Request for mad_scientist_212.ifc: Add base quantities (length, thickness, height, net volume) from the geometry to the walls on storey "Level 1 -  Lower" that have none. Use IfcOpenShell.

First a look at what the model holds.

```python
import ifcopenshell
import ifcopenshell.util.element
import ifcopenshell.util.unit

model = ifcopenshell.open("mad_scientist_212.ifc")
print(model.schema)
for unit_type in ("LENGTHUNIT", "AREAUNIT", "VOLUMEUNIT"):
    print(unit_type, ifcopenshell.util.unit.calculate_unit_scale(model, unit_type))
storey = next(s for s in model.by_type("IfcBuildingStorey") if s.Name == "Level 1 -  Lower")
walls = [e for e in ifcopenshell.util.element.get_decomposition(storey) if e.is_a("IfcWall")]
for e in sorted(walls, key=lambda e: e.id()):
    print(e.id(), e.is_a(), e.Name, list(ifcopenshell.util.element.get_psets(e, qtos_only=True)), sep=" | ")
```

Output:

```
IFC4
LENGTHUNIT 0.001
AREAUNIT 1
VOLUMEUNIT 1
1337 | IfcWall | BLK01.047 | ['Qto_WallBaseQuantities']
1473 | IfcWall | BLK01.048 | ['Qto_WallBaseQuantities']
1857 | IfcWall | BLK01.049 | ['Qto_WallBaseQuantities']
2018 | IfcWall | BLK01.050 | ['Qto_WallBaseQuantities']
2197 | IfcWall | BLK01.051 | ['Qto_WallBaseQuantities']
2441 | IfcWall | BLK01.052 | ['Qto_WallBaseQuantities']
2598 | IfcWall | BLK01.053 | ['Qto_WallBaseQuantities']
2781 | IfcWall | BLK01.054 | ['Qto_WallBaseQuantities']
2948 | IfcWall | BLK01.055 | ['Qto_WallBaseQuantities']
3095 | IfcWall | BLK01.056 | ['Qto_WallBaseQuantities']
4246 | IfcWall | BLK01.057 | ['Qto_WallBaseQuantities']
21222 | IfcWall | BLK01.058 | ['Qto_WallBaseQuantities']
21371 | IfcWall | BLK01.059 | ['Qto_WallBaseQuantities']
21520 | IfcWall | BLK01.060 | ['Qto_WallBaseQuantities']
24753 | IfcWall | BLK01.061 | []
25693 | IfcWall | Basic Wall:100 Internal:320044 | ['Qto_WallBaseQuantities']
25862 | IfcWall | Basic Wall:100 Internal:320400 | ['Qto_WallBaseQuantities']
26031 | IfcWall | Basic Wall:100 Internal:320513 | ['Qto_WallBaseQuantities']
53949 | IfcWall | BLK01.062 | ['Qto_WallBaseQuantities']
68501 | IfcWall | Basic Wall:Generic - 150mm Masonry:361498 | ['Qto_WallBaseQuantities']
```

```python
import ifcopenshell
import ifcopenshell.api.pset
import ifcopenshell.geom
import ifcopenshell.util.element
import ifcopenshell.util.shape
import ifcopenshell.util.unit

model = ifcopenshell.open("mad_scientist_212.ifc")
unit_scale = ifcopenshell.util.unit.calculate_unit_scale(model)
volume_scale = ifcopenshell.util.unit.calculate_unit_scale(model, "VOLUMEUNIT")
settings = ifcopenshell.geom.settings()

storey = next(s for s in model.by_type("IfcBuildingStorey") if s.Name == "Level 1 -  Lower")
walls = [e for e in ifcopenshell.util.element.get_decomposition(storey) if e.is_a("IfcWall")]

for e in sorted(walls, key=lambda e: e.id()):
    if ifcopenshell.util.element.get_psets(e, qtos_only=True, should_inherit=False):
        continue
    # Geometry comes back in metres, in the element's own axes.
    shape = ifcopenshell.geom.create_shape(settings, e)
    values = {
        "Length": ifcopenshell.util.shape.get_x(shape.geometry) / unit_scale,
        "Width": ifcopenshell.util.shape.get_y(shape.geometry) / unit_scale,
        "Height": ifcopenshell.util.shape.get_z(shape.geometry) / unit_scale,
        "NetVolume": ifcopenshell.util.shape.get_volume(shape.geometry) / volume_scale,
    }
    qto = ifcopenshell.api.pset.add_qto(model, product=e, name="Qto_WallBaseQuantities")
    ifcopenshell.api.pset.edit_qto(model, qto=qto, properties=values)
    print(e.id(), {k: round(v, 3) for k, v in values.items()})

model.write("mad_scientist_212-out.ifc")
```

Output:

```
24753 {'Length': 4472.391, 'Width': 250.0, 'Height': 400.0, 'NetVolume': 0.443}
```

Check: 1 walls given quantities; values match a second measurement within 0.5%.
